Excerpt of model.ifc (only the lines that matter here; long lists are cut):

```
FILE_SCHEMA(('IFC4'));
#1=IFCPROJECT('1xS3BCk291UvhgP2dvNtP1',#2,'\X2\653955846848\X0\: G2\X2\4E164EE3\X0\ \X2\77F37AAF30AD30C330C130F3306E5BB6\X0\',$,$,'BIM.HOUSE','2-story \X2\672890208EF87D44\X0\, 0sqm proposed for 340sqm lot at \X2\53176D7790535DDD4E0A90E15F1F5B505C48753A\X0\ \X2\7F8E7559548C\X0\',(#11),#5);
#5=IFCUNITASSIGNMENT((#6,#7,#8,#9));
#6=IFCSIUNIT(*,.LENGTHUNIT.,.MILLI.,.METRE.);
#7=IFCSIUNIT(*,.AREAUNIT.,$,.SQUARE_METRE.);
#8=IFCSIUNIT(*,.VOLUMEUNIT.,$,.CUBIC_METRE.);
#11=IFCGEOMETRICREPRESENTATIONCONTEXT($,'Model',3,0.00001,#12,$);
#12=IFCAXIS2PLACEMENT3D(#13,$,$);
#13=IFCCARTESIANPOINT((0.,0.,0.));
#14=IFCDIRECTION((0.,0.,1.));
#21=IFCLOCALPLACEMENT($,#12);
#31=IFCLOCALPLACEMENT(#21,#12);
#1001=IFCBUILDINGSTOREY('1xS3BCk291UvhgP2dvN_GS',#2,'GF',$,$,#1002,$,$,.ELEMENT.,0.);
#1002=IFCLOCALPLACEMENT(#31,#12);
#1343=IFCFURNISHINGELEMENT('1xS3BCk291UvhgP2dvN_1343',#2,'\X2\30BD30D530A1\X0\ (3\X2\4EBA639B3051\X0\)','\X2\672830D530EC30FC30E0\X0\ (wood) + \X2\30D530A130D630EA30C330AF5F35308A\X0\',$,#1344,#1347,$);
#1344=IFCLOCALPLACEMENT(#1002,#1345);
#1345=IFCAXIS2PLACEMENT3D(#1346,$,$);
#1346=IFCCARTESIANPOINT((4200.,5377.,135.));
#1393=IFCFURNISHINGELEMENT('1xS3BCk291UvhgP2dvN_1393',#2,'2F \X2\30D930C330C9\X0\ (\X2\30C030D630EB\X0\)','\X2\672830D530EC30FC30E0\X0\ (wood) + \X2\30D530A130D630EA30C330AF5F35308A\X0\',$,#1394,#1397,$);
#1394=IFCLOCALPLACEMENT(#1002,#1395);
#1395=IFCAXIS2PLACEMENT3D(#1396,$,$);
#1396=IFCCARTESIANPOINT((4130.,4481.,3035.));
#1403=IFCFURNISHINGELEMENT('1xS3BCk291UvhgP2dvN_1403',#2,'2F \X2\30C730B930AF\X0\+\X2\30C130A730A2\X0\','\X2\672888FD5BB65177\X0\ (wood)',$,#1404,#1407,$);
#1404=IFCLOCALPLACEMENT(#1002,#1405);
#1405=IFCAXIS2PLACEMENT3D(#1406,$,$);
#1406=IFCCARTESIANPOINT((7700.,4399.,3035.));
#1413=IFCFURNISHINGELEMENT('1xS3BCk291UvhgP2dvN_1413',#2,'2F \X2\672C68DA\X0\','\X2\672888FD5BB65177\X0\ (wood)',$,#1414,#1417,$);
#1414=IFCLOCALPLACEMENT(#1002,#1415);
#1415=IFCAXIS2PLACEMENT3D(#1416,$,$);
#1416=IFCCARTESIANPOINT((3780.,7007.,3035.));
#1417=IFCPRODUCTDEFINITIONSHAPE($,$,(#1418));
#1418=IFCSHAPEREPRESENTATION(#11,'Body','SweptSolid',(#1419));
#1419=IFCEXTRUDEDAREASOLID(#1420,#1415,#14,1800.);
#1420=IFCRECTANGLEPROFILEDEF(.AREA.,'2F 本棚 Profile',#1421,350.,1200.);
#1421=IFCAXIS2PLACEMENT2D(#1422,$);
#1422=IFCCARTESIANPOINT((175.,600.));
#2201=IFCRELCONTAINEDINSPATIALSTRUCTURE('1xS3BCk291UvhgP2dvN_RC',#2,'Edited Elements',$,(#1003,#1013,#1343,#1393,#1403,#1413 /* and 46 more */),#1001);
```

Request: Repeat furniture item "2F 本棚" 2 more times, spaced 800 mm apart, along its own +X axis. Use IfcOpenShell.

```python
import ifcopenshell
import ifcopenshell.api.geometry
import ifcopenshell.api.root
import ifcopenshell.util.element
import ifcopenshell.util.placement
import ifcopenshell.util.unit

model = ifcopenshell.open("model.ifc")
unit_scale = ifcopenshell.util.unit.calculate_unit_scale(model)


def reuse_history(source, copy):
    """copy_class also copies each property set's owner history, people and application; keep the originals."""
    for rel in copy.IsDefinedBy:
        if rel.is_a("IfcRelDefinesByProperties") and (history := rel.RelatingPropertyDefinition.OwnerHistory):
            rel.RelatingPropertyDefinition.OwnerHistory = source.OwnerHistory
            ifcopenshell.util.element.remove_deep2(model, history)


source = model.by_guid("1xS3BCk291UvhgP2dvN_1413")
base = ifcopenshell.util.placement.get_local_placement(source.ObjectPlacement)
step = base[:3, 0] * 0.8 / unit_scale

for i in range(1, 3):
    copy = ifcopenshell.api.root.copy_class(model, product=source)
    copy.Representation = ifcopenshell.util.element.copy_deep(
        model, source.Representation, exclude=["IfcGeometricRepresentationContext", "IfcRepresentationMap"]
    )
    reuse_history(source, copy)
    matrix = base.copy()
    matrix[:3, 3] += i * step
    print("added at", matrix[:3, 3].round(3) + 0.0)
    ifcopenshell.api.geometry.edit_object_placement(model, product=copy, matrix=matrix, is_si=False)

model.write("model_rev.ifc")
```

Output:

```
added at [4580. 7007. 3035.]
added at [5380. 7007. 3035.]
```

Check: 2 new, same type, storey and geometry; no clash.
